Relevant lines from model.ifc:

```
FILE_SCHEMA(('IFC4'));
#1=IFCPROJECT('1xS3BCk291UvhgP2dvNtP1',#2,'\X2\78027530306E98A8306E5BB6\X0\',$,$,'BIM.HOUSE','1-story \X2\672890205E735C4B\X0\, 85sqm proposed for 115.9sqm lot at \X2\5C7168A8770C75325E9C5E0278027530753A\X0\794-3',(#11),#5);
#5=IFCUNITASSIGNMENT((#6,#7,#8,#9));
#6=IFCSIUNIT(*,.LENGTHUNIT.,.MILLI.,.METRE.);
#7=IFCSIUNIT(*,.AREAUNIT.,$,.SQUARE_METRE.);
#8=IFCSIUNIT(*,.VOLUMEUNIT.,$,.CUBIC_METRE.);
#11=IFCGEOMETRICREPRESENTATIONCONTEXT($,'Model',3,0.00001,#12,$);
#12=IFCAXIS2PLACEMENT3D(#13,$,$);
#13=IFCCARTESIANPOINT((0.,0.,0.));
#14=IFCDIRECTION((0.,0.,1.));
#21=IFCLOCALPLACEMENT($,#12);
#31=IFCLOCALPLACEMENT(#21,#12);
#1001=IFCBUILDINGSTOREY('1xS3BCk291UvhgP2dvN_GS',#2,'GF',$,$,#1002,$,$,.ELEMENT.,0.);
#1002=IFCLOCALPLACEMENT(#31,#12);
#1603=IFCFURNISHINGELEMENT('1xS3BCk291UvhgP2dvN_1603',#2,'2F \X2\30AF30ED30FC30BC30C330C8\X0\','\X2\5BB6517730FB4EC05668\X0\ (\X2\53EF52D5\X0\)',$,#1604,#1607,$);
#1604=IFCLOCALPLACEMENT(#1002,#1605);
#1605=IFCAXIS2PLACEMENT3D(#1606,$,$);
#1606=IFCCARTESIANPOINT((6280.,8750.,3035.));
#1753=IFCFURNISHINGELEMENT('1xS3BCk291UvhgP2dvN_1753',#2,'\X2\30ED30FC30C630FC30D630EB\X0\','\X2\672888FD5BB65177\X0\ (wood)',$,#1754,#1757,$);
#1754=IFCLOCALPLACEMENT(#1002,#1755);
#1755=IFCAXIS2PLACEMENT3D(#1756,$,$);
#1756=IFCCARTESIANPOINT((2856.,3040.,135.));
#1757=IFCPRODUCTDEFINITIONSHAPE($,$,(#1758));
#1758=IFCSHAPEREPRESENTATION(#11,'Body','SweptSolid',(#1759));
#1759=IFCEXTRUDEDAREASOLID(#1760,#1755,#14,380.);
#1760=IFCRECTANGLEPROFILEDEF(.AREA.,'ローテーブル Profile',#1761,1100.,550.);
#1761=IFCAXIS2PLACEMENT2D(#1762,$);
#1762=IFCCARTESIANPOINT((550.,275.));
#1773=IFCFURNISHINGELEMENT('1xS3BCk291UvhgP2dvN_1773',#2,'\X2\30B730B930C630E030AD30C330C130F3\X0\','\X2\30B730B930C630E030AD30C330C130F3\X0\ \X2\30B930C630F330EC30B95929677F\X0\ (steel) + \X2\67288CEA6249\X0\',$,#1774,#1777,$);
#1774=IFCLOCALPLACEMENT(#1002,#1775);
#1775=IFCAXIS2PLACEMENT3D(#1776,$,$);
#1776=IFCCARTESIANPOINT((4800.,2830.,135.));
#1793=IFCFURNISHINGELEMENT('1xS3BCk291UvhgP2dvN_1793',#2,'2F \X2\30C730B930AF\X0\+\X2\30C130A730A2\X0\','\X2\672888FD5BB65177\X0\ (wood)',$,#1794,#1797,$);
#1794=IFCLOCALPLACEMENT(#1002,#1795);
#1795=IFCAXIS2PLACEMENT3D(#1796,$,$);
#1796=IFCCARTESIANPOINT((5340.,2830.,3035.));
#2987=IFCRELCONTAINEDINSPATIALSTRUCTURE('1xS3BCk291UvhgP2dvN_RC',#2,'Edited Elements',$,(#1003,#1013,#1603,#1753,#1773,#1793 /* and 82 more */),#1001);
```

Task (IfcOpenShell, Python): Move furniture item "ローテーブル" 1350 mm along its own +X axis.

```python
import ifcopenshell
import ifcopenshell.api.geometry
import ifcopenshell.util.placement

model = ifcopenshell.open("model.ifc")

item = model.by_id(1753)
matrix = ifcopenshell.util.placement.get_local_placement(item.ObjectPlacement)
matrix[:3, 3] += matrix[:3, 0] * 1350.0
ifcopenshell.api.geometry.edit_object_placement(model, product=item, matrix=matrix, is_si=False)

print(ifcopenshell.util.placement.get_local_placement(item.ObjectPlacement).round(3) + 0.0)

model.write("model_edited.ifc")
```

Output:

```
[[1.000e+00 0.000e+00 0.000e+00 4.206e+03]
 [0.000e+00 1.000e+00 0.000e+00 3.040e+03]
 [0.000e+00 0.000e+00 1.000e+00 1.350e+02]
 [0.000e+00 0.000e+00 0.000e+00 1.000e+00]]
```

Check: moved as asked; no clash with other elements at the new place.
